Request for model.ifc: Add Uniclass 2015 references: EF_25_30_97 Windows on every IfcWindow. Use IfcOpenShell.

First a look at what the model holds.

```python
import ifcopenshell

model = ifcopenshell.open("model.ifc")
print(model.schema)
print("classifications:", [c.Name for c in model.by_type("IfcClassification")])
for ifc_class in ("IfcDoor", "IfcRoof", "IfcStair", "IfcWall", "IfcWindow"):
    print(ifc_class, len(model.by_type(ifc_class)))
```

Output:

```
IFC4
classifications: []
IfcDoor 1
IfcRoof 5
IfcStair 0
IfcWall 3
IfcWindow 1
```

```python
import ifcopenshell
import ifcopenshell.api.classification

model = ifcopenshell.open("model.ifc")

system = ifcopenshell.api.classification.add_classification(model, classification="Uniclass 2015")

codes = {
    "IfcWindow": ("EF_25_30_97", "Windows"),
}
for ifc_class, (code, name) in codes.items():
    products = model.by_type(ifc_class)
    ifcopenshell.api.classification.add_reference(
        model, products=products, classification=system, identification=code, name=name
    )
    print(code, len(products))

model.write("model_rev.ifc")
```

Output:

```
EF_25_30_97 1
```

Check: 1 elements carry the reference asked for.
